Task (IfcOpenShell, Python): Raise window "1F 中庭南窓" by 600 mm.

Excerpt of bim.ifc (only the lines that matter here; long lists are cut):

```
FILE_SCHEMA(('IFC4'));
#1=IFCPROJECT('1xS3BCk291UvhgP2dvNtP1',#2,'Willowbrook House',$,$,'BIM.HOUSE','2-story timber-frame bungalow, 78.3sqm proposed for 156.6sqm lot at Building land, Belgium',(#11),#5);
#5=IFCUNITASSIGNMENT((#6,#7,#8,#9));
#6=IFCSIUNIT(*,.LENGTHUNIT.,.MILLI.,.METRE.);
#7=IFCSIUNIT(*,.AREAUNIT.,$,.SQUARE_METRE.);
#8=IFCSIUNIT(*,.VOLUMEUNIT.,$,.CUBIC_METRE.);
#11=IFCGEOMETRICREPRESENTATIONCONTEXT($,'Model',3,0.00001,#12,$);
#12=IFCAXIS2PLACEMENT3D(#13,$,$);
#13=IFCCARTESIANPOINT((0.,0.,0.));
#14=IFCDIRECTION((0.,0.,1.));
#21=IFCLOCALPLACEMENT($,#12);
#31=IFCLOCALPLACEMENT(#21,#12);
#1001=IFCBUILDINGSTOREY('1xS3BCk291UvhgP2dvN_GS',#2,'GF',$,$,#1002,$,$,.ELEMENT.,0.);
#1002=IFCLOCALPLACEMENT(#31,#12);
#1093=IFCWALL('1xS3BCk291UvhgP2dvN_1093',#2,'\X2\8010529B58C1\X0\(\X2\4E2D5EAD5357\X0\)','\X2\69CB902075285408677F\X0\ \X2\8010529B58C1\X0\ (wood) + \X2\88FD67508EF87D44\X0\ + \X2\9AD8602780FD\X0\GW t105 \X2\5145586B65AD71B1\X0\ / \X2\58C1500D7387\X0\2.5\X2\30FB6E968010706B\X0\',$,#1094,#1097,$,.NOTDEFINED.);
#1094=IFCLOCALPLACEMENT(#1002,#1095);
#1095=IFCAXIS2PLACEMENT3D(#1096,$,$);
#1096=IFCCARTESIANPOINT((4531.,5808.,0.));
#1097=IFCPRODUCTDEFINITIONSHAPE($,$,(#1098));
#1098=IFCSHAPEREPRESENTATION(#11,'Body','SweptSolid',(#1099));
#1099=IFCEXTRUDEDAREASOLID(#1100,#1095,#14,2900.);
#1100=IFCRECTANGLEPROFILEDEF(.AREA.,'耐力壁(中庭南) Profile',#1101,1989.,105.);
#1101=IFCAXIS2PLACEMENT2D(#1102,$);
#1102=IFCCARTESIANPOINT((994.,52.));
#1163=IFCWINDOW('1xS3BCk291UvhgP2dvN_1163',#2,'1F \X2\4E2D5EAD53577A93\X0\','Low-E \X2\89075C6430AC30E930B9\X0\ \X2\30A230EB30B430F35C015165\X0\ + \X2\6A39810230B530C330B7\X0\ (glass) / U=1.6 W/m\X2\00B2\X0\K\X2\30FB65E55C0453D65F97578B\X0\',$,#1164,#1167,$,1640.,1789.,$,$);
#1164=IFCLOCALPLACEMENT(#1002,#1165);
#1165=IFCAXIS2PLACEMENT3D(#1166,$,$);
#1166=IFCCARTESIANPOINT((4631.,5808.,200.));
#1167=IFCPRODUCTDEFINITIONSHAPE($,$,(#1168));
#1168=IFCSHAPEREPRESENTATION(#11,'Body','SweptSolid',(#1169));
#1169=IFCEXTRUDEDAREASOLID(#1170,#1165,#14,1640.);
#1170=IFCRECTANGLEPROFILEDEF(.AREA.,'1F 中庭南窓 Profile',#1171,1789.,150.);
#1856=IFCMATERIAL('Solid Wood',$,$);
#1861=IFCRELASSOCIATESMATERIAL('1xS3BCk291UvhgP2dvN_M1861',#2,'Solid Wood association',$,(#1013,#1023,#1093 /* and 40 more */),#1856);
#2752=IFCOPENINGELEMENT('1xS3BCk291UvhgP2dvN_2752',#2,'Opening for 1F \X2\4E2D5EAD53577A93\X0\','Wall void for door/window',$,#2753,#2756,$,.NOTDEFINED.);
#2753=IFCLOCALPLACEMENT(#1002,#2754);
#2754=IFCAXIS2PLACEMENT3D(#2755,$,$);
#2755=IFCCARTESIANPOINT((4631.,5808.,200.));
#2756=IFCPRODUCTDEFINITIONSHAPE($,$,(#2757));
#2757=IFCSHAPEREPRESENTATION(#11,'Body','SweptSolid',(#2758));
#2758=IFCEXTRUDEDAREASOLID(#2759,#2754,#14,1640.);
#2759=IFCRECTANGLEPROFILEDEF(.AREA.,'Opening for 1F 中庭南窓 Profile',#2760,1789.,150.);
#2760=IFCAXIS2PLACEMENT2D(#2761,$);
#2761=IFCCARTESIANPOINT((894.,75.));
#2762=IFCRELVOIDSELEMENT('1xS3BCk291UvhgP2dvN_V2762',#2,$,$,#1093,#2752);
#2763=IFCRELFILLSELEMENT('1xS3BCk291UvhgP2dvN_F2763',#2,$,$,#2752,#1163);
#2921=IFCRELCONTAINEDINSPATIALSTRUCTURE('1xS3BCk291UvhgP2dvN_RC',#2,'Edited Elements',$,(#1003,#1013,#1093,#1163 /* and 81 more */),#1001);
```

```python
import numpy as np
import ifcopenshell
import ifcopenshell.api.geometry
import ifcopenshell.util.placement
import ifcopenshell.util.unit

model = ifcopenshell.open("bim.ifc")
unit_scale = ifcopenshell.util.unit.calculate_unit_scale(model)

window = model.by_guid("1xS3BCk291UvhgP2dvN_1163")
opening = window.FillsVoids[0].RelatingOpeningElement
dz = 0.6 / unit_scale

shift = np.array([0.0, 0.0, dz])
# The window is not placed relative to its opening, so move both.
for product in (opening, window):
    matrix = ifcopenshell.util.placement.get_local_placement(product.ObjectPlacement)
    matrix[:3, 3] += shift
    ifcopenshell.api.geometry.edit_object_placement(model, product=product, matrix=matrix, is_si=False)

print(f"moved by {dz * unit_scale:+.3f} m")

model.write("bim-out.ifc")
```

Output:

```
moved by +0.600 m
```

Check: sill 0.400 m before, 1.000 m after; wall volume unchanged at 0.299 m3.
